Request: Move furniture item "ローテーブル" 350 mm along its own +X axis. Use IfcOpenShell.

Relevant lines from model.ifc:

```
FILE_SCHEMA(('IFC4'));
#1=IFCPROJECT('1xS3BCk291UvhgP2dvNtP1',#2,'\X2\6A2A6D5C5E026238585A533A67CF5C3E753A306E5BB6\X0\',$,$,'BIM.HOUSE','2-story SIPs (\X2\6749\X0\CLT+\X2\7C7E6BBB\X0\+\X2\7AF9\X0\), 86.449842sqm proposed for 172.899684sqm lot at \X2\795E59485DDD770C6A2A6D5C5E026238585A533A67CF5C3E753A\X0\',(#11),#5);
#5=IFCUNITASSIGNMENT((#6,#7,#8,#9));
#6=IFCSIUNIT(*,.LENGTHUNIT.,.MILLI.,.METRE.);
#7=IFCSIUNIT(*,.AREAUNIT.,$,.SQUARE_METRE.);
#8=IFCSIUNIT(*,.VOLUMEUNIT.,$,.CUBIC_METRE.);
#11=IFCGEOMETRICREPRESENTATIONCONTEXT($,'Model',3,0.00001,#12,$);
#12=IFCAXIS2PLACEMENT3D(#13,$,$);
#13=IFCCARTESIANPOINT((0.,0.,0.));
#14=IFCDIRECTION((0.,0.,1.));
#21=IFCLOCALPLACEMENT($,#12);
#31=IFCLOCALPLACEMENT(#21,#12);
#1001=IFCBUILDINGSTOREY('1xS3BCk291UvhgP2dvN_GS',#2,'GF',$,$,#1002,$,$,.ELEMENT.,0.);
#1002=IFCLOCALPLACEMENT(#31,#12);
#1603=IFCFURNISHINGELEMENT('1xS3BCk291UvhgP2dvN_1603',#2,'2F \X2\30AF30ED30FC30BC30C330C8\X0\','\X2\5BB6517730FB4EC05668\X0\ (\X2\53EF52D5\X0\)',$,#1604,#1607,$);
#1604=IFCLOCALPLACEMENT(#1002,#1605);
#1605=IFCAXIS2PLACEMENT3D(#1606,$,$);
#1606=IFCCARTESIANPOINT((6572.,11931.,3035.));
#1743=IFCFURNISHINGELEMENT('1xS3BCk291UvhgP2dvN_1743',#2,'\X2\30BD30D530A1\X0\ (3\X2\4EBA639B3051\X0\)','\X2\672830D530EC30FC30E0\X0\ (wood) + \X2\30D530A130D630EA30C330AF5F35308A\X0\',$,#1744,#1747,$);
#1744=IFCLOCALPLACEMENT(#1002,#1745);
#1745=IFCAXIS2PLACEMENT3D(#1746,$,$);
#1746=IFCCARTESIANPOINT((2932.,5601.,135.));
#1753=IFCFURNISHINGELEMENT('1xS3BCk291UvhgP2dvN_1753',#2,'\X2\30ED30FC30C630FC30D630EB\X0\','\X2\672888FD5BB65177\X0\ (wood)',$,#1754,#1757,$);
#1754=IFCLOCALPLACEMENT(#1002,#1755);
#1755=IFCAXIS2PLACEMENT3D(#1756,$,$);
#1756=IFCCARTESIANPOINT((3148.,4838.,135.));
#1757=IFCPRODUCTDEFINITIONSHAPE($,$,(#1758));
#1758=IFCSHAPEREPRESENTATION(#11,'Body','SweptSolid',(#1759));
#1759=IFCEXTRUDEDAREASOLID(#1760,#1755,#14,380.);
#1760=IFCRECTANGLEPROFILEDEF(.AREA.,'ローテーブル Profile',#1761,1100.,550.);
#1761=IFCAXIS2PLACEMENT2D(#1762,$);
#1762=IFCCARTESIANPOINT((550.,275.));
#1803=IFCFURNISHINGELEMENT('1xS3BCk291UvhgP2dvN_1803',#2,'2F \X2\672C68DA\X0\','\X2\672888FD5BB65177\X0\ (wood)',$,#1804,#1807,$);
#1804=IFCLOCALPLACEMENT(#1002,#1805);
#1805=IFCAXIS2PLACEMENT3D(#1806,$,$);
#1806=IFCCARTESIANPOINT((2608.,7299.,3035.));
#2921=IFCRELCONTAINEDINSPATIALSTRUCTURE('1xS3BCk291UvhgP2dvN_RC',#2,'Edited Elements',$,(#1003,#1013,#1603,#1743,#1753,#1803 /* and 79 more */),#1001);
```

```python
import ifcopenshell
import ifcopenshell.api.geometry
import ifcopenshell.util.placement
import ifcopenshell.util.unit

model = ifcopenshell.open("model.ifc")
unit_scale = ifcopenshell.util.unit.calculate_unit_scale(model)

item = model.by_guid("1xS3BCk291UvhgP2dvN_1753")
matrix = ifcopenshell.util.placement.get_local_placement(item.ObjectPlacement)
matrix[:3, 3] += matrix[:3, 0] * 0.35 / unit_scale
ifcopenshell.api.geometry.edit_object_placement(model, product=item, matrix=matrix, is_si=False)

print(ifcopenshell.util.placement.get_local_placement(item.ObjectPlacement).round(3) + 0.0)

model.write("model_updated.ifc")
```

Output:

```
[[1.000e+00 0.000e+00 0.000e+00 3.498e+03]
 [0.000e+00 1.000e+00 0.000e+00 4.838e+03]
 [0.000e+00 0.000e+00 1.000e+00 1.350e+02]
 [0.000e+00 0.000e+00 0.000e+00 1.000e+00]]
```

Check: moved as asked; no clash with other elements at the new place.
